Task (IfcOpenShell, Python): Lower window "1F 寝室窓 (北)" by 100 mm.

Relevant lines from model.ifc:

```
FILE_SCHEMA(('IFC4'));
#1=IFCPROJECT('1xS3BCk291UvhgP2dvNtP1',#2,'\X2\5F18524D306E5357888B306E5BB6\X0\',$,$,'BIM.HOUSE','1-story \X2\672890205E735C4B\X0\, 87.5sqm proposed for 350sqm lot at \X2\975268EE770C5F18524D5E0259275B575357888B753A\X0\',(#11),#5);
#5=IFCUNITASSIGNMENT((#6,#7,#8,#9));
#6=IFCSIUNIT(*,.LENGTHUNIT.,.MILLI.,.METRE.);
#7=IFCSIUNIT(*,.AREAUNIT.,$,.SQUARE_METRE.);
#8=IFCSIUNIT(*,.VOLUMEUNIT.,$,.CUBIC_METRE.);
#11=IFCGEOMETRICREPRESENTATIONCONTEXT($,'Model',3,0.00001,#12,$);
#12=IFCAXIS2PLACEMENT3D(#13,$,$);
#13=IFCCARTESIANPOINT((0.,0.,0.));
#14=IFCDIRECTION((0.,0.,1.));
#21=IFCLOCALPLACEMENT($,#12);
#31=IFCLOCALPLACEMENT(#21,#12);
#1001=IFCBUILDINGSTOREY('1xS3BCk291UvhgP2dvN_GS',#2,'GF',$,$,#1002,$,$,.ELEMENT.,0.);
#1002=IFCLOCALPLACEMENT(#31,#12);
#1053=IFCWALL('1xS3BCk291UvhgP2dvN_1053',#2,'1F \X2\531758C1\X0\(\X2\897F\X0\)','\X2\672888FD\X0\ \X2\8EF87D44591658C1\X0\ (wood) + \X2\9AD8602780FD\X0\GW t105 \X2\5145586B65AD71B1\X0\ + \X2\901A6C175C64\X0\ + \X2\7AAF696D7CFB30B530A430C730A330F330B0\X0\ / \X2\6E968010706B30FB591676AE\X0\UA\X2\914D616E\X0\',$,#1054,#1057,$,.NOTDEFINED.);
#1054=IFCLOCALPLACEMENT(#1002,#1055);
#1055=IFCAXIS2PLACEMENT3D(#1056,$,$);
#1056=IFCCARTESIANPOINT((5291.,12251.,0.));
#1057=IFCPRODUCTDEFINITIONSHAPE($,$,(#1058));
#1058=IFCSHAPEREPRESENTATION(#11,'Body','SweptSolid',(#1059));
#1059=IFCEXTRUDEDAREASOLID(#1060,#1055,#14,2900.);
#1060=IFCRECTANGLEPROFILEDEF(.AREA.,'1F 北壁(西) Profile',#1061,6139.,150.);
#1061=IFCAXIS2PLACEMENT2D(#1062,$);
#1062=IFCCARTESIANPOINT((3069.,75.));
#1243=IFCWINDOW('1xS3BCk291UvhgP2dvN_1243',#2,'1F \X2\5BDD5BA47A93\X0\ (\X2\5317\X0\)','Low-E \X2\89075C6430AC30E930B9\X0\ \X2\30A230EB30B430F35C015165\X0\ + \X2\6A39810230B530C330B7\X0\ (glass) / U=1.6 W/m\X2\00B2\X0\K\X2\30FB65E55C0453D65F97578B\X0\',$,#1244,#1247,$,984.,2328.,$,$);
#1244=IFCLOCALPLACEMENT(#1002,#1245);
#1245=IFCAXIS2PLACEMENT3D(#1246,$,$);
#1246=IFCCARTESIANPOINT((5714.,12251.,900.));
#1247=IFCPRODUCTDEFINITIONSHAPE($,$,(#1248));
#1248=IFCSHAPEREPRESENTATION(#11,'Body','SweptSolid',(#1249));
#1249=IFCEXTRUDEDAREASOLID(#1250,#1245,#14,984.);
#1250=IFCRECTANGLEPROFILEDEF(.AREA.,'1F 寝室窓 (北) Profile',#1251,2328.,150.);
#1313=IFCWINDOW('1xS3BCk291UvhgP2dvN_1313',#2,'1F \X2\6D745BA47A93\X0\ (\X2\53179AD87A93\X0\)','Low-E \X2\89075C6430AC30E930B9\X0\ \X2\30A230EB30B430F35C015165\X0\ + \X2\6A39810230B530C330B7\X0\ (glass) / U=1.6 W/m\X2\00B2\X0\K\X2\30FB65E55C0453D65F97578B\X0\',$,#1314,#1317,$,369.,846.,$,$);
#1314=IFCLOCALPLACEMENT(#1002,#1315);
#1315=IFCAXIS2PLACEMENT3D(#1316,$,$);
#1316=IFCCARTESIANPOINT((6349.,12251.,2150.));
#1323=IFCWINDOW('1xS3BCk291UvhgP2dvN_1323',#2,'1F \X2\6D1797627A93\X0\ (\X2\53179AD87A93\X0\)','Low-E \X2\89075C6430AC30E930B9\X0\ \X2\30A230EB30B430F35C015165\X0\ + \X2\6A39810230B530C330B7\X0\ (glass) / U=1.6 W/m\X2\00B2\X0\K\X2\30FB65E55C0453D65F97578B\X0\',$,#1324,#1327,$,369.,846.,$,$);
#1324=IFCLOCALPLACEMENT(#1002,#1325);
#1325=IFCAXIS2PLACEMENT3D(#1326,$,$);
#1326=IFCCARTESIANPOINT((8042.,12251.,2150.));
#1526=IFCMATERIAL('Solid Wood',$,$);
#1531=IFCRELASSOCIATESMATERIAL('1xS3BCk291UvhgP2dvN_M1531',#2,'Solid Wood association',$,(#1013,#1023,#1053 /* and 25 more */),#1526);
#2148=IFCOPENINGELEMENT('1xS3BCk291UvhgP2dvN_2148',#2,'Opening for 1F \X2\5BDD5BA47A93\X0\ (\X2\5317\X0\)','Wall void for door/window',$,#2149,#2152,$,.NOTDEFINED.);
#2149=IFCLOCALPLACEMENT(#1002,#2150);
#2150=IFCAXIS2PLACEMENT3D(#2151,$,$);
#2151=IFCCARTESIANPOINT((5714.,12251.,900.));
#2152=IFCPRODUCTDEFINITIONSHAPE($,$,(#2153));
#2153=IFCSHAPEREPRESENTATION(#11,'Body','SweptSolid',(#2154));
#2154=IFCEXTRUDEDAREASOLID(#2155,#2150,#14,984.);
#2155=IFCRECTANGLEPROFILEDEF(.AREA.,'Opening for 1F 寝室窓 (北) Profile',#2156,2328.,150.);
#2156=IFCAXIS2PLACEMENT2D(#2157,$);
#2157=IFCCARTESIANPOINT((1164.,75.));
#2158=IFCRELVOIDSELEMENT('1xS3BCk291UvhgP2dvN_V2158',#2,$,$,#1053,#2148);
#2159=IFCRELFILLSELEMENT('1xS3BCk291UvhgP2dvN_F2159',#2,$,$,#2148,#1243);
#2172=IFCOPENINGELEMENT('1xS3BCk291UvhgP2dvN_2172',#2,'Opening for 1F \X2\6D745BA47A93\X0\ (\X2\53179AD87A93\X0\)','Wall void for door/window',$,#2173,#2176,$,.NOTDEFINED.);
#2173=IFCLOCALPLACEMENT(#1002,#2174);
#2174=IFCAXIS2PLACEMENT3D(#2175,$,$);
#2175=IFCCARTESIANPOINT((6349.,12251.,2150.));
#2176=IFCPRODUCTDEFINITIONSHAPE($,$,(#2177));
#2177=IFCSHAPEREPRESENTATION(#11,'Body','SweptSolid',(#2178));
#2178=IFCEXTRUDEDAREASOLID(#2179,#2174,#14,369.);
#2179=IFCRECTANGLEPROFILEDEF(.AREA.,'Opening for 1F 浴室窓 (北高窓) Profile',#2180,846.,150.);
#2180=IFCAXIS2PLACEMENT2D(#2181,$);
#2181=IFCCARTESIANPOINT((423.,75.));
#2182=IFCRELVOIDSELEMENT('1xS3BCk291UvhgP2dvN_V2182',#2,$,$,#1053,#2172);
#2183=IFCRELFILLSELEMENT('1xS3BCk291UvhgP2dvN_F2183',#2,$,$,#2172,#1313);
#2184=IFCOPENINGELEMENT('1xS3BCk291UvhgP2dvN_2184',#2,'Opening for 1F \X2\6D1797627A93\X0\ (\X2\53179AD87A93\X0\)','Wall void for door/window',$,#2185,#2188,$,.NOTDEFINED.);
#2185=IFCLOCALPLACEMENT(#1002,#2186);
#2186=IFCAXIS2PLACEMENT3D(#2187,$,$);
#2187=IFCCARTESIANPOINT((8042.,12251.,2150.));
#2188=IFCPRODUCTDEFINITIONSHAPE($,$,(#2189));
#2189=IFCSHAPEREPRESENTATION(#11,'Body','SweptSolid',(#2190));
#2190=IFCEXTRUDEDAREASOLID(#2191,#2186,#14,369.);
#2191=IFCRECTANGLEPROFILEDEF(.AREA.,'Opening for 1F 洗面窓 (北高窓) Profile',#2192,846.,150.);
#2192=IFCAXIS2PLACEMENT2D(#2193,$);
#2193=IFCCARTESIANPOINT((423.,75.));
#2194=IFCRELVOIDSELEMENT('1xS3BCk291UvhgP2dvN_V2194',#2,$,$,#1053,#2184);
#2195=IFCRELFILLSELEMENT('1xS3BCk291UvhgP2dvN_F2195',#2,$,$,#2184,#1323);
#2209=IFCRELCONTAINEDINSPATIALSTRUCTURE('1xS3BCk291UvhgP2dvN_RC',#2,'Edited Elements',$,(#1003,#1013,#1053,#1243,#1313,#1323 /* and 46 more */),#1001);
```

```python
import numpy as np
import ifcopenshell
import ifcopenshell.api.geometry
import ifcopenshell.util.placement
import ifcopenshell.util.unit

model = ifcopenshell.open("model.ifc")
unit_scale = ifcopenshell.util.unit.calculate_unit_scale(model)

window = model.by_guid("1xS3BCk291UvhgP2dvN_1243")
opening = window.FillsVoids[0].RelatingOpeningElement
dz = -100.0

shift = np.array([0.0, 0.0, dz])
# The window is not placed relative to its opening, so move both.
for product in (opening, window):
    matrix = ifcopenshell.util.placement.get_local_placement(product.ObjectPlacement)
    matrix[:3, 3] += shift
    ifcopenshell.api.geometry.edit_object_placement(model, product=product, matrix=matrix, is_si=False)

print(f"moved by {dz * unit_scale:+.3f} m")

model.write("model_edited.ifc")
```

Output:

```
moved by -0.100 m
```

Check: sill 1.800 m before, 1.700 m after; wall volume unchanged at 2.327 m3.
